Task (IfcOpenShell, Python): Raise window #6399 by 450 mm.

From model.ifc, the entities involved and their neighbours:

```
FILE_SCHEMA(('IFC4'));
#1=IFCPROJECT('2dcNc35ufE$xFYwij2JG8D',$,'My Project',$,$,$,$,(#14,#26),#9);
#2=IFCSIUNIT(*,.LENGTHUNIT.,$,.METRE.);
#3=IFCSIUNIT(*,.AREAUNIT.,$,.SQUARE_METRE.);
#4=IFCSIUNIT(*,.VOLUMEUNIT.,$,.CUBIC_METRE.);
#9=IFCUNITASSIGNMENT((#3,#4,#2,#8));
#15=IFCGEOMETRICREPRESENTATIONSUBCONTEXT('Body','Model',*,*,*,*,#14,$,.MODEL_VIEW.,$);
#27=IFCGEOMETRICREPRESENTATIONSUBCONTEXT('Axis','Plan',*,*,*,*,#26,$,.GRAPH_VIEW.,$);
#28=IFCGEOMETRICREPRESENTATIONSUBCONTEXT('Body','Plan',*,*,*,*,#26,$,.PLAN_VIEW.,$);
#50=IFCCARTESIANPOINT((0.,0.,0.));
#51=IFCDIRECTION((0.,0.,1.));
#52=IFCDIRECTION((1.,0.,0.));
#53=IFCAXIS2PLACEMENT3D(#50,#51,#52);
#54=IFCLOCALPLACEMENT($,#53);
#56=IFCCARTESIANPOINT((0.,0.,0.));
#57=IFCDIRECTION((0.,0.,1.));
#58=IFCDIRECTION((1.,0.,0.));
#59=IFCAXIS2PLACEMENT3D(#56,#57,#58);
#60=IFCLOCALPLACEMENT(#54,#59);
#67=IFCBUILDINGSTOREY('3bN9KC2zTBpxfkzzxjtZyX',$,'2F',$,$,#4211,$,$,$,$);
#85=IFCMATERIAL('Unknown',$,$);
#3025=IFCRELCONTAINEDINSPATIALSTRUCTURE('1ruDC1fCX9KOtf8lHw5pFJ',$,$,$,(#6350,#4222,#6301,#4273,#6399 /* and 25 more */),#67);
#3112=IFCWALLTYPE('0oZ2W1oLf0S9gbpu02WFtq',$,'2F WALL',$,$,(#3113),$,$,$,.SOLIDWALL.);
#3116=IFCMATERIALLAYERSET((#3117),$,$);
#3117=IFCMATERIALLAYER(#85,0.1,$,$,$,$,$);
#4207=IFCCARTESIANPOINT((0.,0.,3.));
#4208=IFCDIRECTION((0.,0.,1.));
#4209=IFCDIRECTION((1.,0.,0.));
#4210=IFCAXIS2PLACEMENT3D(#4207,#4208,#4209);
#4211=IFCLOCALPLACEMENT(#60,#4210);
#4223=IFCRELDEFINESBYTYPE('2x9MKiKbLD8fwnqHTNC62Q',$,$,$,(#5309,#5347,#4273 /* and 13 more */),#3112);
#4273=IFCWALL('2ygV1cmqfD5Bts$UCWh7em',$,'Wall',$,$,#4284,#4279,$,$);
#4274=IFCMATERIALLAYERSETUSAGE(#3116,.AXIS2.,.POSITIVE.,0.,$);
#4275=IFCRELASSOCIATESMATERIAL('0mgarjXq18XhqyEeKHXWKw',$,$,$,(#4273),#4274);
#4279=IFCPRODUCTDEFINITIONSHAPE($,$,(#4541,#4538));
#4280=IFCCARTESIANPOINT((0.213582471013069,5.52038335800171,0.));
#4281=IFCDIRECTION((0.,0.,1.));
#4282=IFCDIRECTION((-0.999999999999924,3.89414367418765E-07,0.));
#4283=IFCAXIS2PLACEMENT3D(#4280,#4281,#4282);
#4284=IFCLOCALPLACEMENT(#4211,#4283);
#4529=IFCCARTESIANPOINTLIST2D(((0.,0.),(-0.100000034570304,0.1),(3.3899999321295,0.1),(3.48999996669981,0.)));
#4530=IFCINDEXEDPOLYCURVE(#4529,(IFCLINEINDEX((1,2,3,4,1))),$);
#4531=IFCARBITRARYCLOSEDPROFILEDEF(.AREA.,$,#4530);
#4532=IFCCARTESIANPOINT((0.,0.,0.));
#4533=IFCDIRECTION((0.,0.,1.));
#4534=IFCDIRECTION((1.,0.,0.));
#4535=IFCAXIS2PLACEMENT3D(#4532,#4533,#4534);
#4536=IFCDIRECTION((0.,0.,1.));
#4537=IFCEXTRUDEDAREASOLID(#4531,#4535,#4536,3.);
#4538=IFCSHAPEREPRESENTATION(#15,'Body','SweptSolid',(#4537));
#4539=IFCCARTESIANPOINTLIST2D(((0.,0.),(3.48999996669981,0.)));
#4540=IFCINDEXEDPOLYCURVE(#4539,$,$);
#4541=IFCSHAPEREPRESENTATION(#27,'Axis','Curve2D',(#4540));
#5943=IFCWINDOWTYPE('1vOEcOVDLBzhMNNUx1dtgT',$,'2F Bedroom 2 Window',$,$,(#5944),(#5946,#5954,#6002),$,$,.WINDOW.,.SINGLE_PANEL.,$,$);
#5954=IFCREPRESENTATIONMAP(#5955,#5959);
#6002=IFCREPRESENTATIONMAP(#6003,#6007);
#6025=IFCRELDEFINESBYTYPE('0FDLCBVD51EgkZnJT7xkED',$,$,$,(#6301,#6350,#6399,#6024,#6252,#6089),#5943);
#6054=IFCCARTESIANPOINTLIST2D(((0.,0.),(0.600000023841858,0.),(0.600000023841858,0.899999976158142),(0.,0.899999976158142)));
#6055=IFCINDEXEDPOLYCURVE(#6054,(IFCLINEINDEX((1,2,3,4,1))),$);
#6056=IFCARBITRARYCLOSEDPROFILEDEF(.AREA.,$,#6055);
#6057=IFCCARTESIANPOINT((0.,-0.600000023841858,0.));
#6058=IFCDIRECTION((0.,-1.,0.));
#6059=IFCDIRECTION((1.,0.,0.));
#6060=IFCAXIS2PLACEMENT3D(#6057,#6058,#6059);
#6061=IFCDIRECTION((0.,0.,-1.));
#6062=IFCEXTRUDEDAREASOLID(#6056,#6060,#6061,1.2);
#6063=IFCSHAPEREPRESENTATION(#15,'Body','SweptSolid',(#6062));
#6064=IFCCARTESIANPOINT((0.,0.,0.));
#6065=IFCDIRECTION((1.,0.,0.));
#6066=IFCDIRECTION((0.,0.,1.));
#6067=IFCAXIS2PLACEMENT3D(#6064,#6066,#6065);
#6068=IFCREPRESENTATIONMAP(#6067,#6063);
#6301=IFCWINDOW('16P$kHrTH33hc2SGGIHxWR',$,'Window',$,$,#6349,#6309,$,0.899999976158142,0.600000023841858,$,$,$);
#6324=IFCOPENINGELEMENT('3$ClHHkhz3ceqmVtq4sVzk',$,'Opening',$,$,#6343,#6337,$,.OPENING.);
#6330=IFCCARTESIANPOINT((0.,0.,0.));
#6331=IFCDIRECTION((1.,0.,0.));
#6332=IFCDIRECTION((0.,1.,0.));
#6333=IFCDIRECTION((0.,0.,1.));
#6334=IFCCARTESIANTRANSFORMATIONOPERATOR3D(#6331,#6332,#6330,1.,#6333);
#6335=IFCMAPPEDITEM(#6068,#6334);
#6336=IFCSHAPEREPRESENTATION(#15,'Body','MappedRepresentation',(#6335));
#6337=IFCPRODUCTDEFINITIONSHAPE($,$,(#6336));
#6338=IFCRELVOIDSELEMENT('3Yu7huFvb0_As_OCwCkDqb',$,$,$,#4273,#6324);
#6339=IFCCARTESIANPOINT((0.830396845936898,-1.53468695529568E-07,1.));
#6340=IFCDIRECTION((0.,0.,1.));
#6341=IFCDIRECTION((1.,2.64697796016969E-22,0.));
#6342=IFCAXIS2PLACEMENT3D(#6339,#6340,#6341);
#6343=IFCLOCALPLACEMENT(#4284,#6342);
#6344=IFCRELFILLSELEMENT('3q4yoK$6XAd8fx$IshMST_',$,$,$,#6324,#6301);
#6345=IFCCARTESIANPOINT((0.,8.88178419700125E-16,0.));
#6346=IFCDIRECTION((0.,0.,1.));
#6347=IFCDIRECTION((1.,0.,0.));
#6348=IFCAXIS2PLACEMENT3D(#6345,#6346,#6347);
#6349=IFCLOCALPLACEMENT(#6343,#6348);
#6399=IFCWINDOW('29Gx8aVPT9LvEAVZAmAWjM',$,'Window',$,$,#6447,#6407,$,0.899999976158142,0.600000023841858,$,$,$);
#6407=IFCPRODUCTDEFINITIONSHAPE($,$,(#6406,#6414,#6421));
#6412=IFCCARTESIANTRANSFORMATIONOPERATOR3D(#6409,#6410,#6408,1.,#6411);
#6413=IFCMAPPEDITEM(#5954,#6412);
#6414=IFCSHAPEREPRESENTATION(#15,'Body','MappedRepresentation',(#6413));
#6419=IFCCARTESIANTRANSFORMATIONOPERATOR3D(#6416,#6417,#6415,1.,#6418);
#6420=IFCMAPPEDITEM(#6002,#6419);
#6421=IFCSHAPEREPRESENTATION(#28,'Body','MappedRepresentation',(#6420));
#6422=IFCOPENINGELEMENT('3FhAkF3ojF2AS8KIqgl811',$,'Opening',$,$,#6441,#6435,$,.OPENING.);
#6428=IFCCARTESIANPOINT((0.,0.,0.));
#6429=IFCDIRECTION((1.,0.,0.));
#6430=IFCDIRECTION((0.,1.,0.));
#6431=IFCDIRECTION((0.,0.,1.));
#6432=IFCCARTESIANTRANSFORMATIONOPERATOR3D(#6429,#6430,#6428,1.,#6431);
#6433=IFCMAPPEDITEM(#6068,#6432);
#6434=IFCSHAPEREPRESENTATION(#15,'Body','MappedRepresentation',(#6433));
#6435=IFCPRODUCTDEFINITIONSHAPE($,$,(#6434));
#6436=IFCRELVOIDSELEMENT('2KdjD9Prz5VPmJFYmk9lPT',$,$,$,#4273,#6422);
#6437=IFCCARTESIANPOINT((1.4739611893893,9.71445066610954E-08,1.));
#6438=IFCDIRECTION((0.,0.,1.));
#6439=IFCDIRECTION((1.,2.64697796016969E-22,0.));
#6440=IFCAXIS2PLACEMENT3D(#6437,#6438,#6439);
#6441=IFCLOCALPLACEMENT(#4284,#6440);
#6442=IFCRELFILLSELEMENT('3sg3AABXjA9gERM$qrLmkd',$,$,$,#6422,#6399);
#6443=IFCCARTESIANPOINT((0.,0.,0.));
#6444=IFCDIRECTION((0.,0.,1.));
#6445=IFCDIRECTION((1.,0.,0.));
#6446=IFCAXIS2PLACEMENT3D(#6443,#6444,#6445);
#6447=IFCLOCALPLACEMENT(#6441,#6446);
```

```python
import numpy as np
import ifcopenshell
import ifcopenshell.api.geometry
import ifcopenshell.util.placement
import ifcopenshell.util.unit

model = ifcopenshell.open("model.ifc")
unit_scale = ifcopenshell.util.unit.calculate_unit_scale(model)

window = model.by_guid("29Gx8aVPT9LvEAVZAmAWjM")
opening = window.FillsVoids[0].RelatingOpeningElement
dz = 0.45 / unit_scale

shift = np.array([0.0, 0.0, dz])
# The window is placed relative to its opening, so it follows when the opening moves.
matrix = ifcopenshell.util.placement.get_local_placement(opening.ObjectPlacement)
matrix[:3, 3] += shift
ifcopenshell.api.geometry.edit_object_placement(
    model, product=opening, matrix=matrix, is_si=False, should_transform_children=True
)

print(f"moved by {dz * unit_scale:+.3f} m")

model.write("model_rev.ifc")
```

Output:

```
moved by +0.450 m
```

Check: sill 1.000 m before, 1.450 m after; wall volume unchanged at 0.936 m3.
